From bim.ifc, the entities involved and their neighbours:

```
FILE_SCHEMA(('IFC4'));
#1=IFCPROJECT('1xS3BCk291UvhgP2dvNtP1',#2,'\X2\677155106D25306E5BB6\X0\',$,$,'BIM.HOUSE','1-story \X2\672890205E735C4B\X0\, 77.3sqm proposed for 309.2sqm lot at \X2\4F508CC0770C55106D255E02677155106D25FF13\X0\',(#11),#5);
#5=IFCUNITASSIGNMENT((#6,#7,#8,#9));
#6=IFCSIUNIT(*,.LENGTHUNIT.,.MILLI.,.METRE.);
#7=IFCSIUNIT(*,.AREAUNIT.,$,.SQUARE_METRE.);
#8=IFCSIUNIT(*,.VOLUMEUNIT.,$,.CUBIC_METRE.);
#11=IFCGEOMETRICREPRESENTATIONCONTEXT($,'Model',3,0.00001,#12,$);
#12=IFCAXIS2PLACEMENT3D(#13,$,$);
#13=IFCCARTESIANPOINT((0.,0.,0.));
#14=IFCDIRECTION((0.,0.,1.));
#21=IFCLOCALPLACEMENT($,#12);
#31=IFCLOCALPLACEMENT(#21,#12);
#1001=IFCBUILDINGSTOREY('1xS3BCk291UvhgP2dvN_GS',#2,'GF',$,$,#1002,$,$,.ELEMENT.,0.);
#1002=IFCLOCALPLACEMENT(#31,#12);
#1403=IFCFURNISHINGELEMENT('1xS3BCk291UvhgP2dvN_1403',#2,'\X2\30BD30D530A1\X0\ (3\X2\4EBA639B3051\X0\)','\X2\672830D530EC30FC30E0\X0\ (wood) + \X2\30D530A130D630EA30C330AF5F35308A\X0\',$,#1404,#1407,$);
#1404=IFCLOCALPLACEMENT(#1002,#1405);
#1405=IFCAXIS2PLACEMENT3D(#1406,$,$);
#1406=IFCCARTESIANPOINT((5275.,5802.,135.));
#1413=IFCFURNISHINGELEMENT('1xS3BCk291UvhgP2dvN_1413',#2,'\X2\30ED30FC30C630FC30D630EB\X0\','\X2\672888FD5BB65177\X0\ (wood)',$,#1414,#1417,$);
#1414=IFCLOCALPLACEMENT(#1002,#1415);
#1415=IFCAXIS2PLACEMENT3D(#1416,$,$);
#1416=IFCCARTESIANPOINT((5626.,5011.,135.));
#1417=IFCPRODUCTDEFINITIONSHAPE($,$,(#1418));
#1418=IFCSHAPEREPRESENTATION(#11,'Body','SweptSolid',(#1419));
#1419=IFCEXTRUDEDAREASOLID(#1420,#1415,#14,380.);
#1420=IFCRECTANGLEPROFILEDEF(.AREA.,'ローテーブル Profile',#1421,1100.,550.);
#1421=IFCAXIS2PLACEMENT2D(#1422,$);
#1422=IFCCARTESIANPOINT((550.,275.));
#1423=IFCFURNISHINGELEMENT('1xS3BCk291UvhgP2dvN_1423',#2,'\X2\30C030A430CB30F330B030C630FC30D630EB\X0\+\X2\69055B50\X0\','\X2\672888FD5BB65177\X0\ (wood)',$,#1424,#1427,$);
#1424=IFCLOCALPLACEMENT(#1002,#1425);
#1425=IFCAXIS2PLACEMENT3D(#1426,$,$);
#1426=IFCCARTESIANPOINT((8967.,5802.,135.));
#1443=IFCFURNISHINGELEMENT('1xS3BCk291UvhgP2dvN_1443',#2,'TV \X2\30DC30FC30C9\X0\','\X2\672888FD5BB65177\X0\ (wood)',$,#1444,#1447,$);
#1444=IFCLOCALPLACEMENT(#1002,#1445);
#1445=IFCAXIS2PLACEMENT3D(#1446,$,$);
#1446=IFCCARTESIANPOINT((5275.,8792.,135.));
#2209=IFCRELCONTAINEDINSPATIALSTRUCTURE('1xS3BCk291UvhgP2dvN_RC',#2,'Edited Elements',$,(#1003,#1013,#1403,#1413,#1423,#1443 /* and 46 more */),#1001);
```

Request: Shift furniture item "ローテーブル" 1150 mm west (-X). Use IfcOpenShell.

```python
import ifcopenshell
import ifcopenshell.api.geometry
import ifcopenshell.util.placement

model = ifcopenshell.open("bim.ifc")

item = model.by_id(1413)
matrix = ifcopenshell.util.placement.get_local_placement(item.ObjectPlacement)
matrix[0, 3] -= 1150.0
ifcopenshell.api.geometry.edit_object_placement(model, product=item, matrix=matrix, is_si=False)

print(ifcopenshell.util.placement.get_local_placement(item.ObjectPlacement).round(3) + 0.0)

model.write("bim-out.ifc")
```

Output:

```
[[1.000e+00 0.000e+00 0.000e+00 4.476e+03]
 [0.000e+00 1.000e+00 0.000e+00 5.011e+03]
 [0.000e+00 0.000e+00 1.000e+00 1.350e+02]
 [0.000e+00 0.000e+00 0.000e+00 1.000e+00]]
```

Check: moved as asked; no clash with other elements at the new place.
